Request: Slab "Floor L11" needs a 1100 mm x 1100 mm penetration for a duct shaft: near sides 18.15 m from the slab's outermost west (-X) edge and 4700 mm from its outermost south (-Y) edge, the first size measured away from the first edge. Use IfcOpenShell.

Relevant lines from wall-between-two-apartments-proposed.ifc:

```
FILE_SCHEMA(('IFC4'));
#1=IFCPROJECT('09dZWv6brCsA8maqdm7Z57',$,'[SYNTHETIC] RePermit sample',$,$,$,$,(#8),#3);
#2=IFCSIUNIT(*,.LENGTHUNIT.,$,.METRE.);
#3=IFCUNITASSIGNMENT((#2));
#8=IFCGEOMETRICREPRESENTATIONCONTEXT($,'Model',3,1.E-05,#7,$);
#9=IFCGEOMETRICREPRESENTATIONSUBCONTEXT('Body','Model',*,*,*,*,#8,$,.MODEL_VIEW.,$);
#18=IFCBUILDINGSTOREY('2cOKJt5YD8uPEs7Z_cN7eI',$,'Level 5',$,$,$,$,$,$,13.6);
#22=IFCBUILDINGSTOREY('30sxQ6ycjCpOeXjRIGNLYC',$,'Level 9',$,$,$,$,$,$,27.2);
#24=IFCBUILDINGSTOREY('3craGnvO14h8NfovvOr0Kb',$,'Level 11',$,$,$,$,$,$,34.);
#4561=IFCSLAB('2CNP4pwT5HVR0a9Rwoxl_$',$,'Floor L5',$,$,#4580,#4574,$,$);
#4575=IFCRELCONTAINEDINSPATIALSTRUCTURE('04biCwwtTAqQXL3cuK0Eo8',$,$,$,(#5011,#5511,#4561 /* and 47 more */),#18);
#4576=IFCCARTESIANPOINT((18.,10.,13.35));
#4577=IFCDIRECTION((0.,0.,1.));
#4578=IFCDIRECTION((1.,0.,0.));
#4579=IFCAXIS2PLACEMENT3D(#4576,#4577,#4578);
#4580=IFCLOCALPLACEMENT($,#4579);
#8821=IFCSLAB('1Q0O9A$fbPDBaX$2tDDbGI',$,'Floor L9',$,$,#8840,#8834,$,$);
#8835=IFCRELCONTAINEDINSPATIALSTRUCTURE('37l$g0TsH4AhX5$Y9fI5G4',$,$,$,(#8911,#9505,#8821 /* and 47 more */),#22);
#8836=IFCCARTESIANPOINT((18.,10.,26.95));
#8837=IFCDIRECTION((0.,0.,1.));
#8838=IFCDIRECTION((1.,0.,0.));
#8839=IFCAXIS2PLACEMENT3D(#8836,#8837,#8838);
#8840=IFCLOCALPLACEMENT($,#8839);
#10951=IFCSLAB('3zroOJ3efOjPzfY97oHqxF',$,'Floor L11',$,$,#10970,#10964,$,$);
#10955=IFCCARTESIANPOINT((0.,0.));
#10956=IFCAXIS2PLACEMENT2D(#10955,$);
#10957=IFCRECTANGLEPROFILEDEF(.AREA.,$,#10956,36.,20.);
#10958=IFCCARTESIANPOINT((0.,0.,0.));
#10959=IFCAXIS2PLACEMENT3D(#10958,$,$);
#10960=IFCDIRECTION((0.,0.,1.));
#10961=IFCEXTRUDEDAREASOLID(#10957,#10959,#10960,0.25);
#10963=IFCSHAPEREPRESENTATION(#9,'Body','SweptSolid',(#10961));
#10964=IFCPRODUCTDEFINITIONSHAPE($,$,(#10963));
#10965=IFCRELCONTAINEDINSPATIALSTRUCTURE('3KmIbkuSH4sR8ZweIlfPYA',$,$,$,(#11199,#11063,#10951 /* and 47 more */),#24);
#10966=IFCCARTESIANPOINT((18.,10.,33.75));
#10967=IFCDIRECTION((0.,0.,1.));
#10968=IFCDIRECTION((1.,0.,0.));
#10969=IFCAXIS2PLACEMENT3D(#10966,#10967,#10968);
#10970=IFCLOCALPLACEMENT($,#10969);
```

```python
import numpy as np
import ifcopenshell
import ifcopenshell.api.feature
import ifcopenshell.api.geometry
import ifcopenshell.api.root
import ifcopenshell.geom
import ifcopenshell.util.placement
import ifcopenshell.util.representation
import ifcopenshell.util.shape
import ifcopenshell.util.unit

model = ifcopenshell.open("wall-between-two-apartments-proposed.ifc")
unit_scale = ifcopenshell.util.unit.calculate_unit_scale(model)
settings = ifcopenshell.geom.settings()


def volume(element):
    """Net volume in cubic metres, openings subtracted."""
    shape = ifcopenshell.geom.create_shape(settings, element)
    return ifcopenshell.util.shape.get_volume(shape.geometry)


slab = model.by_guid("3zroOJ3efOjPzfY97oHqxF")
before = volume(slab)

# Extent in the slab's own axes, in metres. The edges named are its -X and -Y sides.
slab_shape = ifcopenshell.geom.create_shape(settings, slab)
vertices = ifcopenshell.util.shape.get_vertices(slab_shape.geometry)
x_min, y_min, bottom = vertices.min(axis=0)
top = vertices[:, 2].max()

opening = ifcopenshell.api.root.create_entity(model, ifc_class="IfcOpeningElement", name="Duct shaft opening", predefined_type="OPENING")
context = ifcopenshell.util.representation.get_context(model, "Model", "Body", "MODEL_VIEW")
width, depth = 1.1, 1.1
outline = [(0.0, 0.0), (width, 0.0), (width, depth), (0.0, depth), (0.0, 0.0)]
# Overshoot both faces by 50 mm so the cut is clean.
shape = ifcopenshell.api.geometry.add_slab_representation(
    model, context=context, depth=top - bottom + 0.1, polyline=outline
)
ifcopenshell.api.geometry.assign_representation(model, product=opening, representation=shape)

matrix = ifcopenshell.util.placement.get_local_placement(slab.ObjectPlacement)
matrix[:, 3] = matrix @ np.append(np.array([x_min + 18.15, y_min + 4.7, bottom - 0.05]) / unit_scale, 1.0)
ifcopenshell.api.geometry.edit_object_placement(model, product=opening, matrix=matrix, is_si=False)
ifcopenshell.api.feature.add_feature(model, feature=opening, element=slab)

after = volume(slab)

print(f"slab volume {before:.3f} -> {after:.3f} m3")

model.write("wall-between-two-apartments-proposed_updated.ifc")
```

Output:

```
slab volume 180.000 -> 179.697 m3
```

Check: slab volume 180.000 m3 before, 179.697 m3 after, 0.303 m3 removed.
